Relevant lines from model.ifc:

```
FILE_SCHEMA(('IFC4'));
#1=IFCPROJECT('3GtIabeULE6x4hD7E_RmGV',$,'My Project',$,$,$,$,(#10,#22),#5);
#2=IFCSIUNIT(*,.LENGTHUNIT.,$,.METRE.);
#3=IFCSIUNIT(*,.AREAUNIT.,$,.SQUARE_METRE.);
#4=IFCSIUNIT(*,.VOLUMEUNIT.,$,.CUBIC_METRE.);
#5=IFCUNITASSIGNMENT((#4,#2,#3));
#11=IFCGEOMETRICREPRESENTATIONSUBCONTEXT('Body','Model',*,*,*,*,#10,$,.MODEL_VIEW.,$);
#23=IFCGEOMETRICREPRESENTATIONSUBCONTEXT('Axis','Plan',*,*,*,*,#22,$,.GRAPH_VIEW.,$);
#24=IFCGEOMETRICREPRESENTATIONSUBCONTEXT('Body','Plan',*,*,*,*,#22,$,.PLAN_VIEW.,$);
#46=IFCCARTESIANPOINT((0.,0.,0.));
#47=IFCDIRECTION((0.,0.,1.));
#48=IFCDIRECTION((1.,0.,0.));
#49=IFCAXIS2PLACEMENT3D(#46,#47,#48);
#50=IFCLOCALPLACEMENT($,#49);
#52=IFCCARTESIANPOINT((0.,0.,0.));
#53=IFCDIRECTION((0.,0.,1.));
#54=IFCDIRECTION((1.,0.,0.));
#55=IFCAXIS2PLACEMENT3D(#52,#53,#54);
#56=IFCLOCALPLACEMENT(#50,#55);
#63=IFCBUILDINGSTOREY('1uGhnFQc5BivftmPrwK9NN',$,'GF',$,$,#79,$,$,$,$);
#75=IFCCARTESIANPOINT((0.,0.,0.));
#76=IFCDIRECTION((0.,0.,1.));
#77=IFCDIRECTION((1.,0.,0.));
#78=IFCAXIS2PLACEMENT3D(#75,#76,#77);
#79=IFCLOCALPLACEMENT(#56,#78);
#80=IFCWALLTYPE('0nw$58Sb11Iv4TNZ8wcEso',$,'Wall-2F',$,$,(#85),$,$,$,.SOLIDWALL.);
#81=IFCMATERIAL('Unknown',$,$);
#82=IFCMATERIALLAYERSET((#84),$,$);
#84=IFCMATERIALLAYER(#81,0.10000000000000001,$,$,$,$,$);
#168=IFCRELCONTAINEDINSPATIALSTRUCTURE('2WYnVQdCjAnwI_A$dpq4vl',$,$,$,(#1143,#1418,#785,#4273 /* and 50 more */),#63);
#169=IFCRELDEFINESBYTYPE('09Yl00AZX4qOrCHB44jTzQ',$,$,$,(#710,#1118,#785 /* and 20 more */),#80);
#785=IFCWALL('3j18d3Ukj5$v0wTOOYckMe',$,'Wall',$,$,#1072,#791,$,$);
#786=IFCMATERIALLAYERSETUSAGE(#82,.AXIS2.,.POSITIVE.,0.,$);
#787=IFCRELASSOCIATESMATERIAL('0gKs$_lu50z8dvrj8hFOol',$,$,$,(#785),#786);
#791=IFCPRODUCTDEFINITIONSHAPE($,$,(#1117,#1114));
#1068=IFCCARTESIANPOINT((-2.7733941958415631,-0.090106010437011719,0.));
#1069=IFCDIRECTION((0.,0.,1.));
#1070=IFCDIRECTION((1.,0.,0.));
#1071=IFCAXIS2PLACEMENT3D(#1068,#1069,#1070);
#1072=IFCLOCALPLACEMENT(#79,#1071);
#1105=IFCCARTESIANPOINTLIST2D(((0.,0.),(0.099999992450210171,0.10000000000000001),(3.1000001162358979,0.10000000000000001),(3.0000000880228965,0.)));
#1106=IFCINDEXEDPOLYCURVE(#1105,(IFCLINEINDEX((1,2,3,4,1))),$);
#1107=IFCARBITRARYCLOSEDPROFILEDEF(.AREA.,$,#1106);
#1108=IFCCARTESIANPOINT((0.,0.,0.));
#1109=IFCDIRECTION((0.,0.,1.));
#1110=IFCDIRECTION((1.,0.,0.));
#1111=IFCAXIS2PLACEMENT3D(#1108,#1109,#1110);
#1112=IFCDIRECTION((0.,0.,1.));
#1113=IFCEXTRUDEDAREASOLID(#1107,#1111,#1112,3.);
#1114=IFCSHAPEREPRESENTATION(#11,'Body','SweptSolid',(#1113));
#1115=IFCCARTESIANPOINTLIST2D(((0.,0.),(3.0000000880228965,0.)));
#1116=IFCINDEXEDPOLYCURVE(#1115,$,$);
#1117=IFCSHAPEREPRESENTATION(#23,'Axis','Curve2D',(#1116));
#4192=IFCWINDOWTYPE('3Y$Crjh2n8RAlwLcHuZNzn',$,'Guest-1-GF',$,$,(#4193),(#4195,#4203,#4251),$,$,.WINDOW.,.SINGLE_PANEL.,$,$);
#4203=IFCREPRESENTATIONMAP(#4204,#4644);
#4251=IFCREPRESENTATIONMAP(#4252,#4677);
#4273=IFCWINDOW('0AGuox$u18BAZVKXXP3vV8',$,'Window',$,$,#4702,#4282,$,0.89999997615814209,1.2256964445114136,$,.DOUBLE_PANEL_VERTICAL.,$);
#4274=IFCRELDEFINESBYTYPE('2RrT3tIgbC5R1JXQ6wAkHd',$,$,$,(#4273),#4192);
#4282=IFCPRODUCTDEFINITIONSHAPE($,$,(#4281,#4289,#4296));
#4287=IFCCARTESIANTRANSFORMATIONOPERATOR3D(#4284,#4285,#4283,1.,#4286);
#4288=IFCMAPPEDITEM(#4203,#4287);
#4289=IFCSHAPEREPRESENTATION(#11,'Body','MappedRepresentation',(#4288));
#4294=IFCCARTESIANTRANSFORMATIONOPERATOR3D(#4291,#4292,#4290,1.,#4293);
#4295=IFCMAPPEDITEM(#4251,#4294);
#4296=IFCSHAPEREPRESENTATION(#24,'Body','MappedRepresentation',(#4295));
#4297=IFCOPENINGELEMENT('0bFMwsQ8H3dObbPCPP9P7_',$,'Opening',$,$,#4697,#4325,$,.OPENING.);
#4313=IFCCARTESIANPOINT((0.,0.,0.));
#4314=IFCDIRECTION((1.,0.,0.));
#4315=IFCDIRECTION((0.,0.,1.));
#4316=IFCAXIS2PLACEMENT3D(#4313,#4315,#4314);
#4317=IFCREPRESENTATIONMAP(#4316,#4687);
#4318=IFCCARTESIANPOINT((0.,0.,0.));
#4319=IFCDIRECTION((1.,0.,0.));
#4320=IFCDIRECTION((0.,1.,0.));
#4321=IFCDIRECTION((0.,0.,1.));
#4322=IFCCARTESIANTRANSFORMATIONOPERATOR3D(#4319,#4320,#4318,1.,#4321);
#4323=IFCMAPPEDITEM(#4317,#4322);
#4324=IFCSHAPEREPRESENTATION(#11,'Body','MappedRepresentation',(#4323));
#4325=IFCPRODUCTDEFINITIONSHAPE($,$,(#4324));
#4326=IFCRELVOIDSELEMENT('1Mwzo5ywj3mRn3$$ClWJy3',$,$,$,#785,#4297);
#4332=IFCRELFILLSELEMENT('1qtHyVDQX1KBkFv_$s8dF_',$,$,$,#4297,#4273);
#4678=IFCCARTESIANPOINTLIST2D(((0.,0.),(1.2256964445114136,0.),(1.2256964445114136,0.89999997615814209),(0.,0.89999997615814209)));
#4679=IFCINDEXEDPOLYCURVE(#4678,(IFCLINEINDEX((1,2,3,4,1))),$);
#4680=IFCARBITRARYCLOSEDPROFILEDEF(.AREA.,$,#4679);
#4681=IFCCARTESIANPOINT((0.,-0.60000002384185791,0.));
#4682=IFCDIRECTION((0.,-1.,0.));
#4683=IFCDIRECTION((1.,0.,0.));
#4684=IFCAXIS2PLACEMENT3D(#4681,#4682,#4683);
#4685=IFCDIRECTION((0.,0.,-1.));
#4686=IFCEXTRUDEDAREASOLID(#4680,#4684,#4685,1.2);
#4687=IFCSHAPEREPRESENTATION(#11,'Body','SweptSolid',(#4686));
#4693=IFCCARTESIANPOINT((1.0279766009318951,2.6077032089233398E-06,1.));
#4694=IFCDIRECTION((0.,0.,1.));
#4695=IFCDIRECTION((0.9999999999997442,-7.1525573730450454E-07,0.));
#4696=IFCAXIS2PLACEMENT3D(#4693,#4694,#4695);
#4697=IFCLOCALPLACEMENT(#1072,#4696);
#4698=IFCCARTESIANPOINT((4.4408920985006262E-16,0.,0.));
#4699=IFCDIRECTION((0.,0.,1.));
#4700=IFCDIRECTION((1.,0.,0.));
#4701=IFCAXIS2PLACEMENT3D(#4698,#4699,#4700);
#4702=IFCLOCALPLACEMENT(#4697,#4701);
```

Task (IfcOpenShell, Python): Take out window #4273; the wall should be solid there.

```python
import ifcopenshell
import ifcopenshell.api.feature
import ifcopenshell.api.root
import ifcopenshell.geom
import ifcopenshell.util.shape

model = ifcopenshell.open("model.ifc")
settings = ifcopenshell.geom.settings()


def volume(element):
    """Net volume in cubic metres, openings subtracted."""
    shape = ifcopenshell.geom.create_shape(settings, element)
    return ifcopenshell.util.shape.get_volume(shape.geometry)


window = model.by_guid("0AGuox$u18BAZVKXXP3vV8")
opening = window.FillsVoids[0].RelatingOpeningElement
wall = opening.VoidsElements[0].RelatingBuildingElement
before = volume(wall)

ifcopenshell.api.root.remove_product(model, product=window)
ifcopenshell.api.feature.remove_feature(model, feature=opening)

after = volume(wall)

print(f"wall volume {before:.3f} -> {after:.3f} m3")

model.write("model_updated.ifc")
```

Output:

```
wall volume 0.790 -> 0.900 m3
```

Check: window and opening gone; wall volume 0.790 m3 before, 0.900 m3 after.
